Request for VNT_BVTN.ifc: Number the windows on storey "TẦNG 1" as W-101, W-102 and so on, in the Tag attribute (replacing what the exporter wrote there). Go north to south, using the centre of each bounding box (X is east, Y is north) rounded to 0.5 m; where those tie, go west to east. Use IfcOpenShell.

First a look at what the model holds.

```python
import ifcopenshell
import ifcopenshell.util.element
import ifcopenshell.util.placement

model = ifcopenshell.open("VNT_BVTN.ifc")
print(model.schema)
storey = next(s for s in model.by_type("IfcBuildingStorey") if s.Name == "TẦNG 1")
windows = [e for e in ifcopenshell.util.element.get_decomposition(storey) if e.is_a("IfcWindow")]
for e in sorted(windows, key=lambda e: e.id()):
    origin = ifcopenshell.util.placement.get_local_placement(e.ObjectPlacement)[:3, 3]
    print(e.id(), e.Tag, e.Name, origin.round(2) + 0.0, sep=" | ")
```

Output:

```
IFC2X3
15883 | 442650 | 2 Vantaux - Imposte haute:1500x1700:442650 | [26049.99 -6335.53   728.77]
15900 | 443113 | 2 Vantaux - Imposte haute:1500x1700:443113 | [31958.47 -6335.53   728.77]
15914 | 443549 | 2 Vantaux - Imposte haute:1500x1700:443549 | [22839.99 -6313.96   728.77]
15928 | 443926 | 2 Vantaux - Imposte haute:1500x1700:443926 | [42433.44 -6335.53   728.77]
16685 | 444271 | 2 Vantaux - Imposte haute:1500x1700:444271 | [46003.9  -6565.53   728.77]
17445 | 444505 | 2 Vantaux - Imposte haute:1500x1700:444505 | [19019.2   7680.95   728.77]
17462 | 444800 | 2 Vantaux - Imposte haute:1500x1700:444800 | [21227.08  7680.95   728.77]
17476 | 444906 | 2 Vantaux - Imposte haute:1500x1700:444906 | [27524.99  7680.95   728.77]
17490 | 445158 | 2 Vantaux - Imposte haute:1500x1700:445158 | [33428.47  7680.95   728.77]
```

```python
import ifcopenshell
import ifcopenshell.geom
import ifcopenshell.util.element
import ifcopenshell.util.shape

model = ifcopenshell.open("VNT_BVTN.ifc")
settings = ifcopenshell.geom.settings()
settings.set("use-world-coords", True)


def centre(element):
    shape = ifcopenshell.geom.create_shape(settings, element)
    return ifcopenshell.util.shape.get_bbox_centroid(shape.geometry)


storey = next(s for s in model.by_type("IfcBuildingStorey") if s.Name == "TẦNG 1")
windows = [e for e in ifcopenshell.util.element.get_decomposition(storey) if e.is_a("IfcWindow")]

# Insertion points can sit at a corner or the storey origin, so sort by the geometry (in metres).
centres = {e: centre(e) for e in windows}
windows.sort(key=lambda e: (-round(centres[e][1] / 0.5), centres[e][0]))

for i, e in enumerate(windows, start=1):
    number = f"W-1{i:02d}"
    e.Tag = number
    print(e.id(), number)

model.write("VNT_BVTN_edited.ifc")
```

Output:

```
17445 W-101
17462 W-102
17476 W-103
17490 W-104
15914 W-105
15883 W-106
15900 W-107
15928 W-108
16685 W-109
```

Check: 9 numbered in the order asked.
